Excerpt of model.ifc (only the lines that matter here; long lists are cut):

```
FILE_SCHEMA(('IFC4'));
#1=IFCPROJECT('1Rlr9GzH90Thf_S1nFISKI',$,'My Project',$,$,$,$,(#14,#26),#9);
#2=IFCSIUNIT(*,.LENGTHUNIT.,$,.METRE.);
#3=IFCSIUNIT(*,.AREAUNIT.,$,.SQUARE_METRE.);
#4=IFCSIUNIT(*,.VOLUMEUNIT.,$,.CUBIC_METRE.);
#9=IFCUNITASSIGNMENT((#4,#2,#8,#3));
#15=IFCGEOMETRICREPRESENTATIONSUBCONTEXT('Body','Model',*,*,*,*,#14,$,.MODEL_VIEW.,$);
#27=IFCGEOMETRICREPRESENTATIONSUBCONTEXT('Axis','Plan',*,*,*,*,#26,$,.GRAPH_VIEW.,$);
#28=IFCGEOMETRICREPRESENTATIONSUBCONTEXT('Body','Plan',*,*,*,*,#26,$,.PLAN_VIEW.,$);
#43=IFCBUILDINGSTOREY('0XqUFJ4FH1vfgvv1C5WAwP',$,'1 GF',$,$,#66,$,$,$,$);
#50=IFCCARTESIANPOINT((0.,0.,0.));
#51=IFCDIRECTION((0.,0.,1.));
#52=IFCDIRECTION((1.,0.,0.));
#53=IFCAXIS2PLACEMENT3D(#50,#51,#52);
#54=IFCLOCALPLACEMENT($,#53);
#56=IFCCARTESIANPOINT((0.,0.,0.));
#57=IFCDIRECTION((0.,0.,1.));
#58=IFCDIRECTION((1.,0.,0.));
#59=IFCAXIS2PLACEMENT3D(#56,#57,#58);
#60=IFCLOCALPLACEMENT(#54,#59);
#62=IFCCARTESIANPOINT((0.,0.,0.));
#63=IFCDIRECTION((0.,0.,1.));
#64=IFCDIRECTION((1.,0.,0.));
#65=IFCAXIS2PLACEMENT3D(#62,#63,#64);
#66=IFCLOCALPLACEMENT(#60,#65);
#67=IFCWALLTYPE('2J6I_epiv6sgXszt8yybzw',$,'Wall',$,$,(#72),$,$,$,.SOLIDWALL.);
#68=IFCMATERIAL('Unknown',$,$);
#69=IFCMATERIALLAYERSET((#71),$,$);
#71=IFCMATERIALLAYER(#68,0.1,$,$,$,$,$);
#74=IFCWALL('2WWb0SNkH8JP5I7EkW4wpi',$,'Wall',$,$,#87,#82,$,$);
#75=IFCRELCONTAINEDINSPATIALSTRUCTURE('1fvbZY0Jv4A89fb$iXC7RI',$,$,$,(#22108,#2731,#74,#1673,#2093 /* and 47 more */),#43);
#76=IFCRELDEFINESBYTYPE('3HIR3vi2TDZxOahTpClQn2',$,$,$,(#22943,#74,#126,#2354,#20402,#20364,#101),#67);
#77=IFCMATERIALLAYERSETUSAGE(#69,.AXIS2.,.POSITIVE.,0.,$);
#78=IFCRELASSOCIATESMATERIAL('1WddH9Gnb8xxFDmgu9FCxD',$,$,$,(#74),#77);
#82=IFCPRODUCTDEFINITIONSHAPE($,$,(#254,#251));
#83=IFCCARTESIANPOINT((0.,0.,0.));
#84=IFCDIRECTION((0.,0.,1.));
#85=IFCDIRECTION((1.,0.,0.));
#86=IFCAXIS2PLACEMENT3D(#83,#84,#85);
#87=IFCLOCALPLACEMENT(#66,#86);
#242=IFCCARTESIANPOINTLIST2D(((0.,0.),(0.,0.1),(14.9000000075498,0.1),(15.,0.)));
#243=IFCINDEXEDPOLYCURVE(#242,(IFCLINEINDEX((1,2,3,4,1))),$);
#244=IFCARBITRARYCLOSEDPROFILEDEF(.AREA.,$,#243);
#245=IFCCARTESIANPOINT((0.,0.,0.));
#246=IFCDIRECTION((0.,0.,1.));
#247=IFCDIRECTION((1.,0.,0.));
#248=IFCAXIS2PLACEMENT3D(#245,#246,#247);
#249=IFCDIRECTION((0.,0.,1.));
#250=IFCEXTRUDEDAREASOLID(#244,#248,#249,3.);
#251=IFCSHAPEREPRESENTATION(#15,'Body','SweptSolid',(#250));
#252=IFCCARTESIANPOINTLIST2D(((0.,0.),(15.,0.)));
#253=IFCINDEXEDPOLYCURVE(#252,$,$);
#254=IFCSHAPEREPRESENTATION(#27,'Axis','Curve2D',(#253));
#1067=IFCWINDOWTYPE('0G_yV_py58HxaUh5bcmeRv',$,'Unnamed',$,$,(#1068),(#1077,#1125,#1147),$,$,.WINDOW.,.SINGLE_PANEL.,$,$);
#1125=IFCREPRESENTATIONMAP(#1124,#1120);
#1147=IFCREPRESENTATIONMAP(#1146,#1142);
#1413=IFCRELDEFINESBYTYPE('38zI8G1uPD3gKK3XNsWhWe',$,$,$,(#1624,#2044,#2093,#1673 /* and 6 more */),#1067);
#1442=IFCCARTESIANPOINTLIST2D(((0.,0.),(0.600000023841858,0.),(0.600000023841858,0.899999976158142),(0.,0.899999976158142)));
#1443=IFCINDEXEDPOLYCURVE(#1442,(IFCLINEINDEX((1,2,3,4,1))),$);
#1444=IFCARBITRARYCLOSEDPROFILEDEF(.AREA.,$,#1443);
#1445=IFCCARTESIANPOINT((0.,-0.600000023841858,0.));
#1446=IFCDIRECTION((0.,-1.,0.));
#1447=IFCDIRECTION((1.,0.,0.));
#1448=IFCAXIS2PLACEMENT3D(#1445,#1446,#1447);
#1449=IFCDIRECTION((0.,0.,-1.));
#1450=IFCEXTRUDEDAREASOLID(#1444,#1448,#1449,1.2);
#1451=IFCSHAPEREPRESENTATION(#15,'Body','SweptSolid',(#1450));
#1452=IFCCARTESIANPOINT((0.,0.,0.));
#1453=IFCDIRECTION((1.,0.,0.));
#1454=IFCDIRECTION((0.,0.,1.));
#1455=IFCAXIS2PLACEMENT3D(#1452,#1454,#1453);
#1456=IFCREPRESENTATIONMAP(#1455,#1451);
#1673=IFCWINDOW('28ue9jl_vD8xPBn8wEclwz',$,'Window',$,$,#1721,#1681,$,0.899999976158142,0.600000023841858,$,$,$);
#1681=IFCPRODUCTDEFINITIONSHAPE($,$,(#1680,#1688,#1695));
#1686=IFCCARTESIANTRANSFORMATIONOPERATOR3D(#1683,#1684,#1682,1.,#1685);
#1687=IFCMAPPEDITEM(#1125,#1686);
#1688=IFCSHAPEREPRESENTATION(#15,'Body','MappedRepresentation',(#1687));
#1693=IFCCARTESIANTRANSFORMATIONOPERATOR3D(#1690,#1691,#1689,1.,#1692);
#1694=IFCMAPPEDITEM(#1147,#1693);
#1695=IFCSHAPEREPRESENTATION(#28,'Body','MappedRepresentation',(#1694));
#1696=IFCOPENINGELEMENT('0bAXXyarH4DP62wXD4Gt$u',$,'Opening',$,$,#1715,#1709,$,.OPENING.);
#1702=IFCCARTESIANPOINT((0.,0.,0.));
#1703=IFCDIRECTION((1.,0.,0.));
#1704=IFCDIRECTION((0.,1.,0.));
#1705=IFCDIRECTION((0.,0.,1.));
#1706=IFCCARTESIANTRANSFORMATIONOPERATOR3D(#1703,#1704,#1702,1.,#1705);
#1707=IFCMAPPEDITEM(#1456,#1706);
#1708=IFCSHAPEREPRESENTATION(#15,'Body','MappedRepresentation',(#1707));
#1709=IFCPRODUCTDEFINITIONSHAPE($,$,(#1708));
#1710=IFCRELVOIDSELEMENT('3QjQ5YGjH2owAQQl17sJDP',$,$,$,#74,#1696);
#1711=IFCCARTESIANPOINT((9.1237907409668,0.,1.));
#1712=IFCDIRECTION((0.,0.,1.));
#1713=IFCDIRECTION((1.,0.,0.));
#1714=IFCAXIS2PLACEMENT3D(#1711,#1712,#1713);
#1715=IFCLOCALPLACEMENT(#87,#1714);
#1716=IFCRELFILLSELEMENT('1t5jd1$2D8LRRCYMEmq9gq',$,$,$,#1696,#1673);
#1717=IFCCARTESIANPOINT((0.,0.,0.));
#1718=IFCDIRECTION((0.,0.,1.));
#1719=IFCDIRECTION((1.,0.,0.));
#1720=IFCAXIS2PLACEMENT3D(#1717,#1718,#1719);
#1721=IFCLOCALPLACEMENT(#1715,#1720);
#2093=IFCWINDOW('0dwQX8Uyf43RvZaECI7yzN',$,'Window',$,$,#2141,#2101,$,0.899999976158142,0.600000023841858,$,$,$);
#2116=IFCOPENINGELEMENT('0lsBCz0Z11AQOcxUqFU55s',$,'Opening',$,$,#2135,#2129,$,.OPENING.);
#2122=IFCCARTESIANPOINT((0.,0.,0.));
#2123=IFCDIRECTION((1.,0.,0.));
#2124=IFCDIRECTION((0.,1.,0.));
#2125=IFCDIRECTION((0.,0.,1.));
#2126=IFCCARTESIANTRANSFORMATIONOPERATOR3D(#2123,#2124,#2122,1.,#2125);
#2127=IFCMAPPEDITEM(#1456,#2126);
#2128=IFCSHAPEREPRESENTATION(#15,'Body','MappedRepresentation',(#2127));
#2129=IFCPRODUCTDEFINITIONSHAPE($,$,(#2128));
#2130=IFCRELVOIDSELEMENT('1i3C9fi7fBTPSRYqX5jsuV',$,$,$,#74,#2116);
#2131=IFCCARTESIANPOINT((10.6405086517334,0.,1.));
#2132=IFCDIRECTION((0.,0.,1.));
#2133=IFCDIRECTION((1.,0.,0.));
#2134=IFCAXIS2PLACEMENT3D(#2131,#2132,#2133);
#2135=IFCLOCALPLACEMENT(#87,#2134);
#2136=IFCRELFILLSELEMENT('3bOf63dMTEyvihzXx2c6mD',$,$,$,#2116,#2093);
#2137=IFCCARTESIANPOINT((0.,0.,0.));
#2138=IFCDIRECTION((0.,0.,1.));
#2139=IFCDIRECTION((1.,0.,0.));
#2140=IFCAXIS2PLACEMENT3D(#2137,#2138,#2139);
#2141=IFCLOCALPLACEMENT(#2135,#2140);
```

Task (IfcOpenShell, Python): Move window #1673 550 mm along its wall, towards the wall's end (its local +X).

```python
import ifcopenshell
import ifcopenshell.api.geometry
import ifcopenshell.util.placement

model = ifcopenshell.open("model.ifc")

window = model.by_guid("28ue9jl_vD8xPBn8wEclwz")
opening = window.FillsVoids[0].RelatingOpeningElement
wall = opening.VoidsElements[0].RelatingBuildingElement

wall_matrix = ifcopenshell.util.placement.get_local_placement(wall.ObjectPlacement)
shift = wall_matrix[:3, 0] * 0.55
before = ifcopenshell.util.placement.get_local_placement(window.ObjectPlacement)[:3, 3].copy()

# The window is placed relative to its opening, so it follows when the opening moves.
matrix = ifcopenshell.util.placement.get_local_placement(opening.ObjectPlacement)
matrix[:3, 3] += shift
ifcopenshell.api.geometry.edit_object_placement(
    model, product=opening, matrix=matrix, is_si=False, should_transform_children=True
)

after = ifcopenshell.util.placement.get_local_placement(window.ObjectPlacement)[:3, 3]
print("window moved by", (after - before).round(3) + 0.0)

model.write("model_edited.ifc")
```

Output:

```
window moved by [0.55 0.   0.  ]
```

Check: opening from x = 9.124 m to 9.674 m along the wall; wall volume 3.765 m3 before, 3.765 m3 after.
